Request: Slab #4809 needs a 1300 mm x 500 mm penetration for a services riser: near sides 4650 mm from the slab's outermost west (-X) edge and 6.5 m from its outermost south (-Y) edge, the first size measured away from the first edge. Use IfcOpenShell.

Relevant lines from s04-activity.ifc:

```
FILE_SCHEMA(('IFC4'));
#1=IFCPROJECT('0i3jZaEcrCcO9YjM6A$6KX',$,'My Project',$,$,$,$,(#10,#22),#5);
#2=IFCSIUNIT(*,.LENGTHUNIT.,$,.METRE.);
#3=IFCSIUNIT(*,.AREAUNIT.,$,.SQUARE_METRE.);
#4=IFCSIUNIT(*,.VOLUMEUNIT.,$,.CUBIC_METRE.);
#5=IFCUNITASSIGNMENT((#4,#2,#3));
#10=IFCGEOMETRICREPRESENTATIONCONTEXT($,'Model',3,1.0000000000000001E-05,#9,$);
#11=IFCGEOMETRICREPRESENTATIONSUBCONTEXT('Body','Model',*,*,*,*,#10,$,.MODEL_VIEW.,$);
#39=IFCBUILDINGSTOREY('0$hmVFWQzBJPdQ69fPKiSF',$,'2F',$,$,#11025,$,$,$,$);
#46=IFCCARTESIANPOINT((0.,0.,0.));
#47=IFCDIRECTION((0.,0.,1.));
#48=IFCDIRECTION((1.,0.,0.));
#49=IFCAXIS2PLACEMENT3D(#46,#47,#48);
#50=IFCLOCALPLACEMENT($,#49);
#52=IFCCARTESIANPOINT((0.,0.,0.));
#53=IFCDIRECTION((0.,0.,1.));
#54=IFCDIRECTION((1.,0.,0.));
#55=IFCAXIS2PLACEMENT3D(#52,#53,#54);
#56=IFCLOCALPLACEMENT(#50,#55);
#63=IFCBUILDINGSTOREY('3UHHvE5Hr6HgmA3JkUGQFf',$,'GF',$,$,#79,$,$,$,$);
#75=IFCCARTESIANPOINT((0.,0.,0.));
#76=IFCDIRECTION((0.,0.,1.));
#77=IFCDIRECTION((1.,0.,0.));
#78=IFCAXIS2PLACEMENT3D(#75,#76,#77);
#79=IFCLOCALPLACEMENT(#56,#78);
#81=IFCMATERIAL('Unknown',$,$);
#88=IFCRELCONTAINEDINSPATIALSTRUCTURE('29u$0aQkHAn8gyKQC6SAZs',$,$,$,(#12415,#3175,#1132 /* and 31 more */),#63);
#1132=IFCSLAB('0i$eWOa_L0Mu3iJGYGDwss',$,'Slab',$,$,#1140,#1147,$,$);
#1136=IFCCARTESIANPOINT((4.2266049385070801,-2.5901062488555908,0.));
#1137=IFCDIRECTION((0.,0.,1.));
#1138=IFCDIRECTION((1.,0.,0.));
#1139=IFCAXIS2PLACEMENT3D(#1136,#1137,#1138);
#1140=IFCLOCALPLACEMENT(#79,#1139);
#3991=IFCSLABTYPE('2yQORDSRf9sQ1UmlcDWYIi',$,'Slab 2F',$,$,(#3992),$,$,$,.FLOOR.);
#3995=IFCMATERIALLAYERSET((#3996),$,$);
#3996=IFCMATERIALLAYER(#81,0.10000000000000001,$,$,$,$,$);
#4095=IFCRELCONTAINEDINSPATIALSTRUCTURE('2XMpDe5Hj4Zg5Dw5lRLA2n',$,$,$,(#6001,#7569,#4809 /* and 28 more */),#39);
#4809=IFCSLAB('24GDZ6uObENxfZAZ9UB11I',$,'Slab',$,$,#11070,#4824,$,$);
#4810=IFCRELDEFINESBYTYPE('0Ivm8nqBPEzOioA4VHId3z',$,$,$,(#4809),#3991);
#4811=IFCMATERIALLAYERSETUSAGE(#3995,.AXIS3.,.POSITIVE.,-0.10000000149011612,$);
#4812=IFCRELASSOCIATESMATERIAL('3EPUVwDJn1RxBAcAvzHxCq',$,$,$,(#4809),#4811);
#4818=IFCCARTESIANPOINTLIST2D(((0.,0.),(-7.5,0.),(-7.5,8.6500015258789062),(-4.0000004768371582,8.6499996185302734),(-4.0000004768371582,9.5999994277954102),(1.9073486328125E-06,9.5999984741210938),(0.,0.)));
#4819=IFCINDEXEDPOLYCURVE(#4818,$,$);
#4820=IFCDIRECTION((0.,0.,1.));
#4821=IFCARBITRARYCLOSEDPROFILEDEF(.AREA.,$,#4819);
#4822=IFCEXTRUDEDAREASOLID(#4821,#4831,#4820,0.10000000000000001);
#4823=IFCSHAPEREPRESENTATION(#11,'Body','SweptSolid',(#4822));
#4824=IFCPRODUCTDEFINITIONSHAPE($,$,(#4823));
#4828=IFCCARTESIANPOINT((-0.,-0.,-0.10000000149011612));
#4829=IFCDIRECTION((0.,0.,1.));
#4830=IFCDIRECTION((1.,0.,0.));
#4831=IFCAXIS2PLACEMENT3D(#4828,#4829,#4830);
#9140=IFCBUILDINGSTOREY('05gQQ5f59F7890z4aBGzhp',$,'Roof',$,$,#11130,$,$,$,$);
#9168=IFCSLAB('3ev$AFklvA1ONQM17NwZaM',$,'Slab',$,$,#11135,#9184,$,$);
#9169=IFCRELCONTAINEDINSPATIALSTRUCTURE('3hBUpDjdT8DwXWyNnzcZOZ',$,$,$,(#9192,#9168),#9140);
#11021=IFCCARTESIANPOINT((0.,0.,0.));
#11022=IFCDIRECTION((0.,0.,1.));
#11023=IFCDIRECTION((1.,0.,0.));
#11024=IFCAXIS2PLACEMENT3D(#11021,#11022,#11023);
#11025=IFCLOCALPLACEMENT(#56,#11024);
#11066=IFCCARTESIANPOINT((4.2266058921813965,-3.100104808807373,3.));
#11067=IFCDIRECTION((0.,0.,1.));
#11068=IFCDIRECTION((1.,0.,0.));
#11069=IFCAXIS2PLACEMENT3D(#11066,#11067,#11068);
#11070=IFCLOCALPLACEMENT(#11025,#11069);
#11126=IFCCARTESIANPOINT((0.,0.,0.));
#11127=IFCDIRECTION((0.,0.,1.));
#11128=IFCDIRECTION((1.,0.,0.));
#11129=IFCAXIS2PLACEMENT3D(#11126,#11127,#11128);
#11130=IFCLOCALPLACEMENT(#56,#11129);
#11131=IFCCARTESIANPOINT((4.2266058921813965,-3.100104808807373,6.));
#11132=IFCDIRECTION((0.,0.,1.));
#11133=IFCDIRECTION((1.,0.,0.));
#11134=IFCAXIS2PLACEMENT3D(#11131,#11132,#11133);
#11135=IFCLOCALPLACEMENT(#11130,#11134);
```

```python
import numpy as np
import ifcopenshell
import ifcopenshell.api.feature
import ifcopenshell.api.geometry
import ifcopenshell.api.root
import ifcopenshell.geom
import ifcopenshell.util.placement
import ifcopenshell.util.representation
import ifcopenshell.util.shape
import ifcopenshell.util.unit

model = ifcopenshell.open("s04-activity.ifc")
unit_scale = ifcopenshell.util.unit.calculate_unit_scale(model)
settings = ifcopenshell.geom.settings()


def volume(element):
    """Net volume in cubic metres, openings subtracted."""
    shape = ifcopenshell.geom.create_shape(settings, element)
    return ifcopenshell.util.shape.get_volume(shape.geometry)


slab = model.by_guid("24GDZ6uObENxfZAZ9UB11I")
before = volume(slab)

# Extent in the slab's own axes, in metres. The edges named are its -X and -Y sides.
slab_shape = ifcopenshell.geom.create_shape(settings, slab)
vertices = ifcopenshell.util.shape.get_vertices(slab_shape.geometry)
x_min, y_min, bottom = vertices.min(axis=0)
top = vertices[:, 2].max()

opening = ifcopenshell.api.root.create_entity(model, ifc_class="IfcOpeningElement", name="Services riser opening", predefined_type="OPENING")
context = ifcopenshell.util.representation.get_context(model, "Model", "Body", "MODEL_VIEW")
width, depth = 1.3, 0.5
outline = [(0.0, 0.0), (width, 0.0), (width, depth), (0.0, depth), (0.0, 0.0)]
# Overshoot both faces by 50 mm so the cut is clean.
shape = ifcopenshell.api.geometry.add_slab_representation(
    model, context=context, depth=top - bottom + 0.1, polyline=outline
)
ifcopenshell.api.geometry.assign_representation(model, product=opening, representation=shape)

matrix = ifcopenshell.util.placement.get_local_placement(slab.ObjectPlacement)
matrix[:, 3] = matrix @ np.append(np.array([x_min + 4.65, y_min + 6.5, bottom - 0.05]) / unit_scale, 1.0)
ifcopenshell.api.geometry.edit_object_placement(model, product=opening, matrix=matrix, is_si=False)
ifcopenshell.api.feature.add_feature(model, feature=opening, element=slab)

after = volume(slab)

print(f"slab volume {before:.3f} -> {after:.3f} m3")

model.write("s04-activity_v2.ifc")
```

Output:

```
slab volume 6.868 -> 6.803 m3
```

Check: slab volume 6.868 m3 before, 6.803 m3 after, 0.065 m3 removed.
